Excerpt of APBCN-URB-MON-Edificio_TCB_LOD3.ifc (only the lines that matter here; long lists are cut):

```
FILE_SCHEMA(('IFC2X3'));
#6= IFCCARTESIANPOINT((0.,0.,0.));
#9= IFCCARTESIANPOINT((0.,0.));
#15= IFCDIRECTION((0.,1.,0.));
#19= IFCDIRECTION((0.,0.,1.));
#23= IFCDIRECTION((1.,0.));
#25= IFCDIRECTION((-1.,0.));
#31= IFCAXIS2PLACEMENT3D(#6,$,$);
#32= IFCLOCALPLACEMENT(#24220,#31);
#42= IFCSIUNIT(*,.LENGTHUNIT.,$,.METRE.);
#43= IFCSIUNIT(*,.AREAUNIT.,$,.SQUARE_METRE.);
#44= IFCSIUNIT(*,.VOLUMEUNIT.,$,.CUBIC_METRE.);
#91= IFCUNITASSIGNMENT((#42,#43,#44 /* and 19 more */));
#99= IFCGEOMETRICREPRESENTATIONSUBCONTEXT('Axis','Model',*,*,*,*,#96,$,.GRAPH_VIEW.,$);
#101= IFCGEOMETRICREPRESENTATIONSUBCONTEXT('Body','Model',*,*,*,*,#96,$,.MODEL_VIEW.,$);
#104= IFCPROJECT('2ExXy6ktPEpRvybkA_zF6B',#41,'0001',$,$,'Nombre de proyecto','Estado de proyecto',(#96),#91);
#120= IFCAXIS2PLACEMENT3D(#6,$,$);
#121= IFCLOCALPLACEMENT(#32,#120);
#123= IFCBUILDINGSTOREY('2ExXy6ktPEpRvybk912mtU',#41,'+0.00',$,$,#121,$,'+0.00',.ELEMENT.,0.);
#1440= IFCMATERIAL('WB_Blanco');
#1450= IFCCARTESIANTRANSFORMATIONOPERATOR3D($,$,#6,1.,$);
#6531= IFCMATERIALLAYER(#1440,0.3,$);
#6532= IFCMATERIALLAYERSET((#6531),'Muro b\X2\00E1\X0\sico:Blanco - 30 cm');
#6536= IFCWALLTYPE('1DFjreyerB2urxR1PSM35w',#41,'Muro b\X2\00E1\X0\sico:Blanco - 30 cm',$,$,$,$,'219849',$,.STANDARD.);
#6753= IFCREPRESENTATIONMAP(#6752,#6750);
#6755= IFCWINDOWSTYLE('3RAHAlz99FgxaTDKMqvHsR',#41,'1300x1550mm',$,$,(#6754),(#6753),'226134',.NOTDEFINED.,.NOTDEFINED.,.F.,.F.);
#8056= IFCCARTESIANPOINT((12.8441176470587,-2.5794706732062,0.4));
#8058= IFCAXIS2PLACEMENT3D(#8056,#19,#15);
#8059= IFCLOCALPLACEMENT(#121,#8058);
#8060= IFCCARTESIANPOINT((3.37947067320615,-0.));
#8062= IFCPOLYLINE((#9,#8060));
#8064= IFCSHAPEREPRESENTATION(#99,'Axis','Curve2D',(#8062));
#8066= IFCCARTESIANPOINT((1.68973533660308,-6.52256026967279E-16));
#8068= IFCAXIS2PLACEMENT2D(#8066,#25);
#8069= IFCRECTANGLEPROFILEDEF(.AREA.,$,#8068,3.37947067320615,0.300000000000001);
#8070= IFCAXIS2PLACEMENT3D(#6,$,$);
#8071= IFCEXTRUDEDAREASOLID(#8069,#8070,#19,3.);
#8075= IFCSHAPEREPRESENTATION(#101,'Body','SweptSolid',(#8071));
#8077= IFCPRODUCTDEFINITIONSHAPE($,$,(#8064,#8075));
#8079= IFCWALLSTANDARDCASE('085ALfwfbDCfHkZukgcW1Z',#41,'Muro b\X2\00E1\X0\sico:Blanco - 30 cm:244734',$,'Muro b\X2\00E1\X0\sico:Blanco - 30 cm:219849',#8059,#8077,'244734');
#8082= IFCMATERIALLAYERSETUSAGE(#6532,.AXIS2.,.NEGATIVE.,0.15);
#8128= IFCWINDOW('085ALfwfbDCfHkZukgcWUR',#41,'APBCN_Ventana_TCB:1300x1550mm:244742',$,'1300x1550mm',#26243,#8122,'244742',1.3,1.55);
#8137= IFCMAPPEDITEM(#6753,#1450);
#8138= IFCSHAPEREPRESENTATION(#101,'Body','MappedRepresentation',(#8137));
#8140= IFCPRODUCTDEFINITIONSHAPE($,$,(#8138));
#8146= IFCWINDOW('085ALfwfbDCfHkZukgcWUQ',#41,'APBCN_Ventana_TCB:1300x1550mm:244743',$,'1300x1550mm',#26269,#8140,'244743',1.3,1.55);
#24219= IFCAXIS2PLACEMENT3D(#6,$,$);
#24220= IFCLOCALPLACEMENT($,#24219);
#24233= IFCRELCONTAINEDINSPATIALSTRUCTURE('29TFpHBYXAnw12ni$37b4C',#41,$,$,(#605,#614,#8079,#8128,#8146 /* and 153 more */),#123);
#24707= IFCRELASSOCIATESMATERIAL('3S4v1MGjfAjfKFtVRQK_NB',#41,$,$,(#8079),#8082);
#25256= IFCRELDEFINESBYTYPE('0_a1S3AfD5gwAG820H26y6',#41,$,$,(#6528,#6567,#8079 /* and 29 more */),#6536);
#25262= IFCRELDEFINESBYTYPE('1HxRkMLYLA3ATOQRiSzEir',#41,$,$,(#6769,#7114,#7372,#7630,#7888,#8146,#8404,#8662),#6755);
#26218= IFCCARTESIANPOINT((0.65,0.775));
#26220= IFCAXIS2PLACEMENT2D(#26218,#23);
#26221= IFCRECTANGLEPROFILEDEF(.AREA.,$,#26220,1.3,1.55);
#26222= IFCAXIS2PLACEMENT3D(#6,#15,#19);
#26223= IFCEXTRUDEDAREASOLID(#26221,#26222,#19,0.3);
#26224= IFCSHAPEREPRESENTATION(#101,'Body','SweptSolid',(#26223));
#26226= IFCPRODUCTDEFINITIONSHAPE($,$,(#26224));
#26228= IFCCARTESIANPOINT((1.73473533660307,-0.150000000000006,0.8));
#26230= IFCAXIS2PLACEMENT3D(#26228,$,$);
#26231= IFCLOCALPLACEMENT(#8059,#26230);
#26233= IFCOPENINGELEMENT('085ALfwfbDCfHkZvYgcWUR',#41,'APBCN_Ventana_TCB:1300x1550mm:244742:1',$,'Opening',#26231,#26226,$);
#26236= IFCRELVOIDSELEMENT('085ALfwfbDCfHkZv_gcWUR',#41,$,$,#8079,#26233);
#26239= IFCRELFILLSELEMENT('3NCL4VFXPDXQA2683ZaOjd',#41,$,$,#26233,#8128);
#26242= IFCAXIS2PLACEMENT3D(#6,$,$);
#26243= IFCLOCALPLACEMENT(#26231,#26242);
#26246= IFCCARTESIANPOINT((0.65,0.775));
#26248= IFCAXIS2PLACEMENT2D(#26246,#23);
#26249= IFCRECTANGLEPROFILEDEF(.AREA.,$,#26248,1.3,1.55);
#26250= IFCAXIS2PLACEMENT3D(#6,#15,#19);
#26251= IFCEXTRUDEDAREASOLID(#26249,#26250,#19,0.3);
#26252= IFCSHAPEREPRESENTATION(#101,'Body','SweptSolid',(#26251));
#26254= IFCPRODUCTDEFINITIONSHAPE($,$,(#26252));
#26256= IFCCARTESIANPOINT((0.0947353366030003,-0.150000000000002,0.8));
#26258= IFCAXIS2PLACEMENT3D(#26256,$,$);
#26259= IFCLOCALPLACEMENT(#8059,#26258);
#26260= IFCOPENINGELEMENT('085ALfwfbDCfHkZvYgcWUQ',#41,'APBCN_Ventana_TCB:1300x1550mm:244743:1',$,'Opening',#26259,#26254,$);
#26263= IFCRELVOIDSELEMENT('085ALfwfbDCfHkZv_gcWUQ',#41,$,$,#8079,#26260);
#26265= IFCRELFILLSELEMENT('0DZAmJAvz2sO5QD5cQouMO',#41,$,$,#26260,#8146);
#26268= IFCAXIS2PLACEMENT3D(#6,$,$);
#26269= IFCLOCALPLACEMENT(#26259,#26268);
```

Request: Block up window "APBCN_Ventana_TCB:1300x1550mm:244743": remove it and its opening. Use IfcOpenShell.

```python
import ifcopenshell
import ifcopenshell.api.feature
import ifcopenshell.api.root
import ifcopenshell.geom
import ifcopenshell.util.shape

model = ifcopenshell.open("APBCN-URB-MON-Edificio_TCB_LOD3.ifc")
settings = ifcopenshell.geom.settings()


def volume(element):
    """Net volume in cubic metres, openings subtracted."""
    shape = ifcopenshell.geom.create_shape(settings, element)
    return ifcopenshell.util.shape.get_volume(shape.geometry)


window = model.by_guid("085ALfwfbDCfHkZukgcWUQ")
opening = window.FillsVoids[0].RelatingOpeningElement
wall = opening.VoidsElements[0].RelatingBuildingElement
before = volume(wall)

ifcopenshell.api.root.remove_product(model, product=window)
ifcopenshell.api.feature.remove_feature(model, feature=opening)

after = volume(wall)

print(f"wall volume {before:.3f} -> {after:.3f} m3")

model.write("APBCN-URB-MON-Edificio_TCB_LOD3_rev.ifc")
```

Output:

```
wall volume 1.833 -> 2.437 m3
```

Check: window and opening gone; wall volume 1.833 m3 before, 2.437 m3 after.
